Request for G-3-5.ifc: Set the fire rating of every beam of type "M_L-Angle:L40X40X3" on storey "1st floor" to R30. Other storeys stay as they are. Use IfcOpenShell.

First a look at what the model holds.

```python
import ifcopenshell
import ifcopenshell.util.element

model = ifcopenshell.open("G-3-5.ifc")
print(model.schema)
storey = next(s for s in model.by_type("IfcBuildingStorey") if s.Name == "1st floor")
beams = [e for e in ifcopenshell.util.element.get_decomposition(storey) if e.is_a("IfcBeam")]
seen = {}
for e in beams:
    element_type = ifcopenshell.util.element.get_type(e)
    key = (element_type.Name if element_type != e and element_type else None, ifcopenshell.util.element.get_pset(e, "Pset_BeamCommon", "FireRating"))
    seen[key] = seen.get(key, 0) + 1
for (name, value), count in sorted(seen.items(), key=str):
    print(count, "x", name, "|", value)
```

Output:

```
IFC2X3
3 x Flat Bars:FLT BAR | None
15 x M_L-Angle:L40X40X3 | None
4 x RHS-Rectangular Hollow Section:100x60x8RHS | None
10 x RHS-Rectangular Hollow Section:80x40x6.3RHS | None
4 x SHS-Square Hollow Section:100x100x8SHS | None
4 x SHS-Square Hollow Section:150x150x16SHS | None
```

```python
import ifcopenshell
import ifcopenshell.api.pset
import ifcopenshell.util.element

model = ifcopenshell.open("G-3-5.ifc")

storey = next(s for s in model.by_type("IfcBuildingStorey") if s.Name == "1st floor")
beams = [e for e in ifcopenshell.util.element.get_decomposition(storey) if e.is_a("IfcBeam")]

count = 0
for e in beams:
    element_type = ifcopenshell.util.element.get_type(e)
    if element_type in (None, e) or element_type.Name != "M_L-Angle:L40X40X3":
        continue
    # add_pset returns the element's existing set when there is one.
    pset = ifcopenshell.api.pset.add_pset(model, product=e, name="Pset_BeamCommon")
    ifcopenshell.api.pset.edit_pset(model, pset=pset, properties={"FireRating": "R30"})
    count += 1

print(count, "beams updated")

model.write("G-3-5-out.ifc")
```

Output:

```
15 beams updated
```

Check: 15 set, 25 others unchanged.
